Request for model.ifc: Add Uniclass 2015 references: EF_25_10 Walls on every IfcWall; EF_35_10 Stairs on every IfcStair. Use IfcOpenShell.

First a look at what the model holds.

```python
import ifcopenshell

model = ifcopenshell.open("model.ifc")
print(model.schema)
print("classifications:", [c.Name for c in model.by_type("IfcClassification")])
for ifc_class in ("IfcDoor", "IfcRoof", "IfcStair", "IfcWall", "IfcWindow"):
    print(ifc_class, len(model.by_type(ifc_class)))
```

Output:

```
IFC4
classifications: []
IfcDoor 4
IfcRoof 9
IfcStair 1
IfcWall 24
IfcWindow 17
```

```python
import ifcopenshell
import ifcopenshell.api.classification

model = ifcopenshell.open("model.ifc")

system = ifcopenshell.api.classification.add_classification(model, classification="Uniclass 2015")

codes = {
    "IfcWall": ("EF_25_10", "Walls"),
    "IfcStair": ("EF_35_10", "Stairs"),
}
for ifc_class, (code, name) in codes.items():
    products = model.by_type(ifc_class)
    ifcopenshell.api.classification.add_reference(
        model, products=products, classification=system, identification=code, name=name
    )
    print(code, len(products))

model.write("model_edited.ifc")
```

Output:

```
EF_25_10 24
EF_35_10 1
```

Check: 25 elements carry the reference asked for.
